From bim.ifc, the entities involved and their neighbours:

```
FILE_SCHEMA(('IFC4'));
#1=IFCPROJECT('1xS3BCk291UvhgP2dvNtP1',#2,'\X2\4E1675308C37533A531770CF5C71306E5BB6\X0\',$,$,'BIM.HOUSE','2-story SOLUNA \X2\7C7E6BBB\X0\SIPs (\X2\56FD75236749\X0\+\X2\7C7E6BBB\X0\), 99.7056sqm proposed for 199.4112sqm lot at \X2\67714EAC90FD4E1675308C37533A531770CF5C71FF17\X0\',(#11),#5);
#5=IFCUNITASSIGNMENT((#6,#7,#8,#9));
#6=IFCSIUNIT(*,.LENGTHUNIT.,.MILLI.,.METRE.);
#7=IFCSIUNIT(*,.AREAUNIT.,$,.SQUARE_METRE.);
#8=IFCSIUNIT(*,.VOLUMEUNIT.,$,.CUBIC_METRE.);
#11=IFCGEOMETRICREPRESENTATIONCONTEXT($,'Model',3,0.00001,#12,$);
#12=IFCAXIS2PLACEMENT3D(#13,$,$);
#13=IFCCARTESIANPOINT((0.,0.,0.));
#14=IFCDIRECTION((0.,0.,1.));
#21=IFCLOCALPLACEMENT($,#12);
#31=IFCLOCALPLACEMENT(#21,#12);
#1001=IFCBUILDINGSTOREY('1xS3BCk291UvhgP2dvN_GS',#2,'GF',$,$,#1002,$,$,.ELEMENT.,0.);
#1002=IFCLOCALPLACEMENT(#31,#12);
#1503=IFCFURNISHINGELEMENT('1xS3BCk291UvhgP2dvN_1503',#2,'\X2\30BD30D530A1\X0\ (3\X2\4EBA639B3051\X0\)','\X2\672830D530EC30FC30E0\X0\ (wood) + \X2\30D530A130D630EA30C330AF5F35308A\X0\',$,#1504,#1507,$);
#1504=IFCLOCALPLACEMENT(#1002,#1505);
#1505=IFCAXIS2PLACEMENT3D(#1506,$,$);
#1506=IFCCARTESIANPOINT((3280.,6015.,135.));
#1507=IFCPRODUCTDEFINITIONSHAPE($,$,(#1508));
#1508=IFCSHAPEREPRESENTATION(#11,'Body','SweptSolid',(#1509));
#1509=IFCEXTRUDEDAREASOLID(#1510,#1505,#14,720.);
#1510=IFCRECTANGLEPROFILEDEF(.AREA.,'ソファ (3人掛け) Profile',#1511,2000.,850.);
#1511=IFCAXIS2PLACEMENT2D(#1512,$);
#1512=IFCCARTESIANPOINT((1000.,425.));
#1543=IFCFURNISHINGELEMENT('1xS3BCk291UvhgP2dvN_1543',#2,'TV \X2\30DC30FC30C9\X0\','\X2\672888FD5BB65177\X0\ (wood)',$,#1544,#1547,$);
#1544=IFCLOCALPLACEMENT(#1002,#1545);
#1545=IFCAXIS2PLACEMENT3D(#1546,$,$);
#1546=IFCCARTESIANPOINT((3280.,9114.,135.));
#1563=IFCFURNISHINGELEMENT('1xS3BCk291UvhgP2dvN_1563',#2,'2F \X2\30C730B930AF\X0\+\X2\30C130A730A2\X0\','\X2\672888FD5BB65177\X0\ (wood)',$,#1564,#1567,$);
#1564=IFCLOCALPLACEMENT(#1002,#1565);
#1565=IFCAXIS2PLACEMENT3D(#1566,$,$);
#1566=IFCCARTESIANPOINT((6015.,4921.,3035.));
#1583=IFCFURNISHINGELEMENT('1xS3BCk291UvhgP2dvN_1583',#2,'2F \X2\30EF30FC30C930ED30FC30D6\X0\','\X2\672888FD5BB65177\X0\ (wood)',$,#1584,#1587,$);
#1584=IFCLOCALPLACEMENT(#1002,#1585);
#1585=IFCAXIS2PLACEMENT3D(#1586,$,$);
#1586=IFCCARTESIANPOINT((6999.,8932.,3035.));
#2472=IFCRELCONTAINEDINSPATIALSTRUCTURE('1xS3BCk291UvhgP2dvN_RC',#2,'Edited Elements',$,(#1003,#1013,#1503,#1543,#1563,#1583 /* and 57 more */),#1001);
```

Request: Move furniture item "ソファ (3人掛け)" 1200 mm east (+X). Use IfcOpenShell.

```python
import ifcopenshell
import ifcopenshell.api.geometry
import ifcopenshell.util.placement

model = ifcopenshell.open("bim.ifc")

item = model.by_id(1503)
matrix = ifcopenshell.util.placement.get_local_placement(item.ObjectPlacement)
matrix[0, 3] += 1200.0
ifcopenshell.api.geometry.edit_object_placement(model, product=item, matrix=matrix, is_si=False)

print(ifcopenshell.util.placement.get_local_placement(item.ObjectPlacement).round(3) + 0.0)

model.write("bim_edited.ifc")
```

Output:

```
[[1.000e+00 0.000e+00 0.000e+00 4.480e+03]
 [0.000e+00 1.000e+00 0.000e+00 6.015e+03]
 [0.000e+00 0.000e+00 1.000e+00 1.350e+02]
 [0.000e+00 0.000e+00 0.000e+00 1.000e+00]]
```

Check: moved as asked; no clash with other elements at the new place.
